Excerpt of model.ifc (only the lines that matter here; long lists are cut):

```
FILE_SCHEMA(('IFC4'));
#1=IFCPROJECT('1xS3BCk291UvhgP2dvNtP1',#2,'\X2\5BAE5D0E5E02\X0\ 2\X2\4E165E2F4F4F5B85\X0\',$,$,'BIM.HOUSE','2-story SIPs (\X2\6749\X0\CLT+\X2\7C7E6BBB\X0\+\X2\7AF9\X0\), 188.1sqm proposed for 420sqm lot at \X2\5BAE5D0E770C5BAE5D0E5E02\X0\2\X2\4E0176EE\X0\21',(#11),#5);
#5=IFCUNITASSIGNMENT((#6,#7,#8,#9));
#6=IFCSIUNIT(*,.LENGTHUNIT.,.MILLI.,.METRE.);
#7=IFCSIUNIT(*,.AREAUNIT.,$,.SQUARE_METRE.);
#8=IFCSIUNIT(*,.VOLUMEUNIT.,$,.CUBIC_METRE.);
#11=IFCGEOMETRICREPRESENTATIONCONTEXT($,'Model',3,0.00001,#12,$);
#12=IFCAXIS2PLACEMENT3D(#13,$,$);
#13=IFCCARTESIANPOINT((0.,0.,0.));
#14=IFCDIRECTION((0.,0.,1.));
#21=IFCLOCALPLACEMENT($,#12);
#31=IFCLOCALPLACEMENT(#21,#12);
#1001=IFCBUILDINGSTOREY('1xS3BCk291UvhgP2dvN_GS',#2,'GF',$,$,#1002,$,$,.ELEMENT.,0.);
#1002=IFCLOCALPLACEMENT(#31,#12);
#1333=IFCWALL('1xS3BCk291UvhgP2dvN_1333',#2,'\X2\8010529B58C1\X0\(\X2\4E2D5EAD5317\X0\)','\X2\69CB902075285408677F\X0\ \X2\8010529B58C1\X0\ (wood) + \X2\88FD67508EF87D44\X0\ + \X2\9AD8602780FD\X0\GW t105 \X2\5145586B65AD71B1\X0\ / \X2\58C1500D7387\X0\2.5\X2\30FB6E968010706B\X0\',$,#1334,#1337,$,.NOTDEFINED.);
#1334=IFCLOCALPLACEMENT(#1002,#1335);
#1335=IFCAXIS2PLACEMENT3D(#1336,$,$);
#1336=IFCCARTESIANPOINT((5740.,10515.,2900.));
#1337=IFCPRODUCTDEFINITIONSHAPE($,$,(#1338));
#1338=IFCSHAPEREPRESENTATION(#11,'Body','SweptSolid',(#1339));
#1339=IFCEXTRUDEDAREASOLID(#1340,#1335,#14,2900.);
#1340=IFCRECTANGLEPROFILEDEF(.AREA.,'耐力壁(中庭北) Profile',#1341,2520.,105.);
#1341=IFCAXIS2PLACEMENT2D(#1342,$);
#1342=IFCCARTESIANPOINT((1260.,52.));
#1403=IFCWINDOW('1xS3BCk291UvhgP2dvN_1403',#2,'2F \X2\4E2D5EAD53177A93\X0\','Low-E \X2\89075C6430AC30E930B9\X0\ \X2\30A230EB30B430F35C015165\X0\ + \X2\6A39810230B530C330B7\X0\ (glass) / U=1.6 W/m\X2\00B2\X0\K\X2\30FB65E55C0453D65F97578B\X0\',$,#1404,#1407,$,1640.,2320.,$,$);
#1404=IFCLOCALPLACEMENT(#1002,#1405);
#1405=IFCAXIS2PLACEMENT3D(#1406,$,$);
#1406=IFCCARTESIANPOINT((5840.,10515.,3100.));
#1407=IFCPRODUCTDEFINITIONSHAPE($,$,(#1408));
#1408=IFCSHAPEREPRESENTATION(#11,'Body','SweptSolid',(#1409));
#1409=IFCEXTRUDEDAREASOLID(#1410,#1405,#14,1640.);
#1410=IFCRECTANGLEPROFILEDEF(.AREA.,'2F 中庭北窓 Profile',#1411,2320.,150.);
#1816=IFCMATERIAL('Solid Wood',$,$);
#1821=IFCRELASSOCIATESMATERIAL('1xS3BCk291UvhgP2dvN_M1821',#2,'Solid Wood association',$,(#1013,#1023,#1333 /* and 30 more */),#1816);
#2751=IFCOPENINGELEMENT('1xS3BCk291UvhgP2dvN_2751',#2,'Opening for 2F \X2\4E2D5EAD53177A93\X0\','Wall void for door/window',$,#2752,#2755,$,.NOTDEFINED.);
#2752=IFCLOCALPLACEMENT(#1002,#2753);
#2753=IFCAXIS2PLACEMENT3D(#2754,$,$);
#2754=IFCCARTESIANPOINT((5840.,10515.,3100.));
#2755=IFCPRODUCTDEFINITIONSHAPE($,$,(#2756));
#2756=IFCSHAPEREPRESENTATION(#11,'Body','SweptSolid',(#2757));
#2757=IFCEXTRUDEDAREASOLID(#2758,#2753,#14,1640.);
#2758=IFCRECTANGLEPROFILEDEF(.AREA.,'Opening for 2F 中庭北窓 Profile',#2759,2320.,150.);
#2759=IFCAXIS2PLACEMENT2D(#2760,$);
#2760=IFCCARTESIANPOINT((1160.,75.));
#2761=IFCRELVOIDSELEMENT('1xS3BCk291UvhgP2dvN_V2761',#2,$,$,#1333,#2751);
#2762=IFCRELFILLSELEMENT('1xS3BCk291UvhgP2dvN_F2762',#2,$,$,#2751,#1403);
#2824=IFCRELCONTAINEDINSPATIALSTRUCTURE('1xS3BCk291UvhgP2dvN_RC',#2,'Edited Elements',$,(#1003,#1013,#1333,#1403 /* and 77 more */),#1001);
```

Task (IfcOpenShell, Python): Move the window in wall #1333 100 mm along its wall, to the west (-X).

```python
import ifcopenshell
import ifcopenshell.api.geometry
import ifcopenshell.util.placement
import ifcopenshell.util.unit

model = ifcopenshell.open("model.ifc")
unit_scale = ifcopenshell.util.unit.calculate_unit_scale(model)

window = model.by_guid("1xS3BCk291UvhgP2dvN_1403")
opening = window.FillsVoids[0].RelatingOpeningElement
wall = opening.VoidsElements[0].RelatingBuildingElement

wall_matrix = ifcopenshell.util.placement.get_local_placement(wall.ObjectPlacement)
shift = wall_matrix[:3, 0] * -0.1 / unit_scale
before = ifcopenshell.util.placement.get_local_placement(window.ObjectPlacement)[:3, 3].copy()

# The window is not placed relative to its opening, so move both.
for product in (opening, window):
    matrix = ifcopenshell.util.placement.get_local_placement(product.ObjectPlacement)
    matrix[:3, 3] += shift
    ifcopenshell.api.geometry.edit_object_placement(model, product=product, matrix=matrix, is_si=False)

after = ifcopenshell.util.placement.get_local_placement(window.ObjectPlacement)[:3, 3]
print("window moved by", (after - before).round(3) + 0.0)

model.write("model_edited.ifc")
```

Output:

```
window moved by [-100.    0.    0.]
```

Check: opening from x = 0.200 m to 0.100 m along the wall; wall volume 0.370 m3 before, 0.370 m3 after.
